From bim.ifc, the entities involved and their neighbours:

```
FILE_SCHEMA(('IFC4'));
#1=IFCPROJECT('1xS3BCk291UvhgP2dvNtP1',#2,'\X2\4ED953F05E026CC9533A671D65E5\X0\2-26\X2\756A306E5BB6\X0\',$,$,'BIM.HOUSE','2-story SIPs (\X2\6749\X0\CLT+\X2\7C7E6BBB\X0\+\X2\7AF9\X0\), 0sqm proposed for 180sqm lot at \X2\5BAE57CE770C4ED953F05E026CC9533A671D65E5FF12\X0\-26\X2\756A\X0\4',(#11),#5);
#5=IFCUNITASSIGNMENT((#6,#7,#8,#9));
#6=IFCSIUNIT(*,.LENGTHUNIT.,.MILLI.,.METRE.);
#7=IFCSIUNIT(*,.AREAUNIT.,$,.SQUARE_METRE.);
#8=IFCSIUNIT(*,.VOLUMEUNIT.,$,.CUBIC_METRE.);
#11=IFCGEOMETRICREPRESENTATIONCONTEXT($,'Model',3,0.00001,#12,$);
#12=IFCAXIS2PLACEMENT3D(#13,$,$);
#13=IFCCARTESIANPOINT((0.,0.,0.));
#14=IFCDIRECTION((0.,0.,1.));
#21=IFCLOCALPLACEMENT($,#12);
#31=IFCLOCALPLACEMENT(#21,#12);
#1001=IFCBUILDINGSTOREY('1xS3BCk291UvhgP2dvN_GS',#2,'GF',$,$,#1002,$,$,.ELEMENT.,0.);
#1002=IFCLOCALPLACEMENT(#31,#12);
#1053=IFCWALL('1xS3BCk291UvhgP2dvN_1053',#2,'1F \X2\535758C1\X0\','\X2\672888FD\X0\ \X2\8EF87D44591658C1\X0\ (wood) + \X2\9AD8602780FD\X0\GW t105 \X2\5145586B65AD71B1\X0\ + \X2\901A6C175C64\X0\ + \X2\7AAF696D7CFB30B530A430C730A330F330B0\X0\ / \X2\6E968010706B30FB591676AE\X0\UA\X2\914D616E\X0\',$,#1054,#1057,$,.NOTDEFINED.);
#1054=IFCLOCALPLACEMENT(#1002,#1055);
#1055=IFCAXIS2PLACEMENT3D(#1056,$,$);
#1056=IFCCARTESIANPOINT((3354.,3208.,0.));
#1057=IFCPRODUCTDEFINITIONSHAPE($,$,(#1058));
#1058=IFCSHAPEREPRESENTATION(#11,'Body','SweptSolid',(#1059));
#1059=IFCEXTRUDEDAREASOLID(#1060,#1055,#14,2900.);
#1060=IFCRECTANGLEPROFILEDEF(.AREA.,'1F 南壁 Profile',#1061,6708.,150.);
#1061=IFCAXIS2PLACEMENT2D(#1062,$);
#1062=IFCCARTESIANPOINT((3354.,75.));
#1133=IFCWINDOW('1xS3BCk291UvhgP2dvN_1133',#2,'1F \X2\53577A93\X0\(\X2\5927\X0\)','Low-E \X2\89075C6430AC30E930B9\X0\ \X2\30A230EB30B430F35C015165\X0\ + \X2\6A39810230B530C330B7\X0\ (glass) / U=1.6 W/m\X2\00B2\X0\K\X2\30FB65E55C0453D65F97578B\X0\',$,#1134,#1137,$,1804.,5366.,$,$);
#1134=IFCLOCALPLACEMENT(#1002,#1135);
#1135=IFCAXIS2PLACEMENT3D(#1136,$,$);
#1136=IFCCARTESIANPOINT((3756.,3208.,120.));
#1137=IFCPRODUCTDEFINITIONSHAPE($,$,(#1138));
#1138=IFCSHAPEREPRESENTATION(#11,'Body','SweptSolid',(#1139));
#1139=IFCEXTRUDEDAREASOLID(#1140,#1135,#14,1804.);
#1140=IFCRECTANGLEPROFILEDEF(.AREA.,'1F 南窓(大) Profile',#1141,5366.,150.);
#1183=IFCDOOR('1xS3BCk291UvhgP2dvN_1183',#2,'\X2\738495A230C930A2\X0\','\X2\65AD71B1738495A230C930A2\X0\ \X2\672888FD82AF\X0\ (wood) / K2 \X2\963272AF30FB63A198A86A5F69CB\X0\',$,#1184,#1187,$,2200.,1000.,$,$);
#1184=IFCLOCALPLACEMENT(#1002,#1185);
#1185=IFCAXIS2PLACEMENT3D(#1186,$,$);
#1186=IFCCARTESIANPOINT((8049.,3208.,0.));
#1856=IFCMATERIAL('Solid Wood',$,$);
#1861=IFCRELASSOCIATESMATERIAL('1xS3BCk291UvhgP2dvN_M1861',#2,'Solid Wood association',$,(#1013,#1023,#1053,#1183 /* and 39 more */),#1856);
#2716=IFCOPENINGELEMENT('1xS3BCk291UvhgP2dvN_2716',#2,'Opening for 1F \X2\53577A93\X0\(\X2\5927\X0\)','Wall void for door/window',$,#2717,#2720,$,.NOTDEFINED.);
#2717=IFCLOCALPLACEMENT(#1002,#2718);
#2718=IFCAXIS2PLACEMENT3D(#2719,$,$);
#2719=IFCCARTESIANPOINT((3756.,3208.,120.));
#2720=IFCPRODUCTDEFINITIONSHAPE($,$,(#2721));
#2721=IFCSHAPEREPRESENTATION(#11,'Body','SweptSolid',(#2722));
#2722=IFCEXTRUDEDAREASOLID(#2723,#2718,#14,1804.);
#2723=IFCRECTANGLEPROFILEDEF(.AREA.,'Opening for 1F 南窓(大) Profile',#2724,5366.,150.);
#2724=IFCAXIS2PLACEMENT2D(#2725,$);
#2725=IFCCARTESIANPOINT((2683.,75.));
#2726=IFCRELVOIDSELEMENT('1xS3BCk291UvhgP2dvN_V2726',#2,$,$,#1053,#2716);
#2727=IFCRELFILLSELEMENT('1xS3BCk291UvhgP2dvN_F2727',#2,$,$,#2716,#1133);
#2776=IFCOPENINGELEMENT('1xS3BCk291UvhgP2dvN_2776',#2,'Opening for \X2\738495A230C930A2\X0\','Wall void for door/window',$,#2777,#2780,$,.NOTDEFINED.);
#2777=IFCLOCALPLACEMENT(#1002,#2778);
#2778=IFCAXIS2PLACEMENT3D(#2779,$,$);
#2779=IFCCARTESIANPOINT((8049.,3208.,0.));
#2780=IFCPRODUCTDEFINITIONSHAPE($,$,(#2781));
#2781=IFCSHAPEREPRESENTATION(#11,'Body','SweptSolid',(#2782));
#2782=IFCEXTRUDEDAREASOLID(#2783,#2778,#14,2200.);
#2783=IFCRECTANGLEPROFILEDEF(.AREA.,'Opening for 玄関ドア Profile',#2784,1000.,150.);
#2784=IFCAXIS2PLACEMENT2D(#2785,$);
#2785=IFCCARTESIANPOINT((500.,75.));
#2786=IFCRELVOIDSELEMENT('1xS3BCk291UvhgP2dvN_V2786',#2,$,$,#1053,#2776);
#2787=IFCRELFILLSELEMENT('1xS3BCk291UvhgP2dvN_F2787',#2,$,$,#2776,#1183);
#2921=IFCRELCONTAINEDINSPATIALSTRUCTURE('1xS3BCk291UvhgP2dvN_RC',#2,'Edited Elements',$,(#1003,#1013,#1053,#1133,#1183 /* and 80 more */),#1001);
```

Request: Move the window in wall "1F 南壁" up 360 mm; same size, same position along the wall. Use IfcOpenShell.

```python
import numpy as np
import ifcopenshell
import ifcopenshell.api.geometry
import ifcopenshell.util.placement
import ifcopenshell.util.unit

model = ifcopenshell.open("bim.ifc")
unit_scale = ifcopenshell.util.unit.calculate_unit_scale(model)

window = model.by_guid("1xS3BCk291UvhgP2dvN_1133")
opening = window.FillsVoids[0].RelatingOpeningElement
dz = 360.0

shift = np.array([0.0, 0.0, dz])
# The window is not placed relative to its opening, so move both.
for product in (opening, window):
    matrix = ifcopenshell.util.placement.get_local_placement(product.ObjectPlacement)
    matrix[:3, 3] += shift
    ifcopenshell.api.geometry.edit_object_placement(model, product=product, matrix=matrix, is_si=False)

print(f"moved by {dz * unit_scale:+.3f} m")

model.write("bim_updated.ifc")
```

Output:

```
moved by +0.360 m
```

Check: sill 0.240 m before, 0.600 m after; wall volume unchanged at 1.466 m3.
